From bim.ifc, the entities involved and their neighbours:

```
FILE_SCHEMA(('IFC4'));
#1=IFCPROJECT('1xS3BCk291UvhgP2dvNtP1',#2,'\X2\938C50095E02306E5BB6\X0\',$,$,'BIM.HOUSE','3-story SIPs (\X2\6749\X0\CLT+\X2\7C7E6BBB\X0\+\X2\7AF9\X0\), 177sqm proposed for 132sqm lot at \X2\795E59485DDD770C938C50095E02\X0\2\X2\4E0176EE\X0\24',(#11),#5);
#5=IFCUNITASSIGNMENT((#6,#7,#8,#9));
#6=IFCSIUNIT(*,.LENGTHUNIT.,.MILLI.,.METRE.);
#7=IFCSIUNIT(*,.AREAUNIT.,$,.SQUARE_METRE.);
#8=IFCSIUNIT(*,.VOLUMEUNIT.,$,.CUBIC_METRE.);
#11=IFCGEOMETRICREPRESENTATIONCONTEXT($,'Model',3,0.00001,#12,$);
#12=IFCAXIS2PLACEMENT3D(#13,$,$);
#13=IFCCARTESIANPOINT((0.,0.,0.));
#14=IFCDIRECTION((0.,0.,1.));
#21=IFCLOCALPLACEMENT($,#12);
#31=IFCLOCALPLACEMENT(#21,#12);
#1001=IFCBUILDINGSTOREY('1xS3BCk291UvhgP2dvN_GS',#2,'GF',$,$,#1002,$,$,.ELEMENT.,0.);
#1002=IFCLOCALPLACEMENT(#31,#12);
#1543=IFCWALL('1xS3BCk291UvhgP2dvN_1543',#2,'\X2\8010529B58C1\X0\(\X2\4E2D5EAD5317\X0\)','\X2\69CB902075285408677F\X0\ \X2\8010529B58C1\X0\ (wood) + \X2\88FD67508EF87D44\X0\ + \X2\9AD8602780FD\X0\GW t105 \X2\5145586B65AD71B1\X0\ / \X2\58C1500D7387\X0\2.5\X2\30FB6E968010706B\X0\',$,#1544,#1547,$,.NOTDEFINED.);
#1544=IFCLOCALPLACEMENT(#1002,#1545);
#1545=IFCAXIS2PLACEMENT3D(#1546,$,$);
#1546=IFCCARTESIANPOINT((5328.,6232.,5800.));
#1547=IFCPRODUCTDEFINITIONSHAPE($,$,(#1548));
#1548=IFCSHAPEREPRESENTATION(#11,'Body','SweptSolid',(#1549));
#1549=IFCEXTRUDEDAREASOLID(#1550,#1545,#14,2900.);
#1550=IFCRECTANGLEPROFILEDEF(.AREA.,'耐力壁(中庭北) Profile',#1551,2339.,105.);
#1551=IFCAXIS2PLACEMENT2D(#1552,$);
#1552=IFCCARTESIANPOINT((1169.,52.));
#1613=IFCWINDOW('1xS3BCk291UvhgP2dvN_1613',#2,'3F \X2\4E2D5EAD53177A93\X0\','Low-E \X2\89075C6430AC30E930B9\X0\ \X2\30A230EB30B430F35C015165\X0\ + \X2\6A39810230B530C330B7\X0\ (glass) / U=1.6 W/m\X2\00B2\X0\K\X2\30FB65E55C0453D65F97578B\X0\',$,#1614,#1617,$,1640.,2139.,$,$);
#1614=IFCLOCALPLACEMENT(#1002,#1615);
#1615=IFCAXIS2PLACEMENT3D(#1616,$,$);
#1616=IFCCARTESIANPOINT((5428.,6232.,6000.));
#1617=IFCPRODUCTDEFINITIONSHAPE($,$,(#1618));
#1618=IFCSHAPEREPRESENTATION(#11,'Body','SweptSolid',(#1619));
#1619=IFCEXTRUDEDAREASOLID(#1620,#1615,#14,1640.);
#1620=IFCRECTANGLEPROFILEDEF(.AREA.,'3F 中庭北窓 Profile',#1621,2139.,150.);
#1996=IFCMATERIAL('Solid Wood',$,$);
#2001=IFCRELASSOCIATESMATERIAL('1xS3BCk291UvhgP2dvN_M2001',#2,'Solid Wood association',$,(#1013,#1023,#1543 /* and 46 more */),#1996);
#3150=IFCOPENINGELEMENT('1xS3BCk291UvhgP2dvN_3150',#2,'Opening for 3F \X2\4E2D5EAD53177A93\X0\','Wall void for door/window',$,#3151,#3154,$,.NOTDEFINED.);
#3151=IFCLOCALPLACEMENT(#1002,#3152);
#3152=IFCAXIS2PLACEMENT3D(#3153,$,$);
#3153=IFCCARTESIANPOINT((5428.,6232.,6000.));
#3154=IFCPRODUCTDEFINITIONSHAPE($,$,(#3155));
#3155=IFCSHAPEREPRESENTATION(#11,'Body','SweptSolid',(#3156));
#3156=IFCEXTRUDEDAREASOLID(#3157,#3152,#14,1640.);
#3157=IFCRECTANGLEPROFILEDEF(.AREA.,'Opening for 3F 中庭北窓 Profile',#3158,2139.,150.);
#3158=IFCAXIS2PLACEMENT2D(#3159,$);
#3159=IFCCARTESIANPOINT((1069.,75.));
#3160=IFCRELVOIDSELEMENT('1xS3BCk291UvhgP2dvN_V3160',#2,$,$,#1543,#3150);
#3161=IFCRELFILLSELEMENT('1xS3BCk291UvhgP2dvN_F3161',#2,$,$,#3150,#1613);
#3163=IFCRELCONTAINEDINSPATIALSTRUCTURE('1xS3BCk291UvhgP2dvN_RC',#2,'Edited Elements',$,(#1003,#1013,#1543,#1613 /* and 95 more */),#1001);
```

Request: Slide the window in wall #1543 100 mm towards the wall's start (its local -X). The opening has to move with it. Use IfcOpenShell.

```python
import ifcopenshell
import ifcopenshell.api.geometry
import ifcopenshell.util.placement
import ifcopenshell.util.unit

model = ifcopenshell.open("bim.ifc")
unit_scale = ifcopenshell.util.unit.calculate_unit_scale(model)

window = model.by_guid("1xS3BCk291UvhgP2dvN_1613")
opening = window.FillsVoids[0].RelatingOpeningElement
wall = opening.VoidsElements[0].RelatingBuildingElement

wall_matrix = ifcopenshell.util.placement.get_local_placement(wall.ObjectPlacement)
shift = wall_matrix[:3, 0] * -0.1 / unit_scale
before = ifcopenshell.util.placement.get_local_placement(window.ObjectPlacement)[:3, 3].copy()

# The window is not placed relative to its opening, so move both.
for product in (opening, window):
    matrix = ifcopenshell.util.placement.get_local_placement(product.ObjectPlacement)
    matrix[:3, 3] += shift
    ifcopenshell.api.geometry.edit_object_placement(model, product=product, matrix=matrix, is_si=False)

after = ifcopenshell.util.placement.get_local_placement(window.ObjectPlacement)[:3, 3]
print("window moved by", (after - before).round(3) + 0.0)

model.write("bim_v2.ifc")
```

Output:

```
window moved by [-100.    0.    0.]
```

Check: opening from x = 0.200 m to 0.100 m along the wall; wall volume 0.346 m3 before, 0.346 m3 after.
